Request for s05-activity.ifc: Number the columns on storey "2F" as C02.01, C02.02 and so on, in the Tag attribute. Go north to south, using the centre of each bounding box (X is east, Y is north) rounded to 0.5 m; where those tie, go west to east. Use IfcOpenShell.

First a look at what the model holds.

```python
import ifcopenshell
import ifcopenshell.util.element
import ifcopenshell.util.placement

model = ifcopenshell.open("s05-activity.ifc")
print(model.schema)
storey = next(s for s in model.by_type("IfcBuildingStorey") if s.Name == "2F")
columns = [e for e in ifcopenshell.util.element.get_decomposition(storey) if e.is_a("IfcColumn")]
for e in sorted(columns, key=lambda e: e.id()):
    origin = ifcopenshell.util.placement.get_local_placement(e.ObjectPlacement)[:3, 3]
    print(e.id(), e.Tag, e.Name, origin.round(2) + 0.0, sep=" | ")
```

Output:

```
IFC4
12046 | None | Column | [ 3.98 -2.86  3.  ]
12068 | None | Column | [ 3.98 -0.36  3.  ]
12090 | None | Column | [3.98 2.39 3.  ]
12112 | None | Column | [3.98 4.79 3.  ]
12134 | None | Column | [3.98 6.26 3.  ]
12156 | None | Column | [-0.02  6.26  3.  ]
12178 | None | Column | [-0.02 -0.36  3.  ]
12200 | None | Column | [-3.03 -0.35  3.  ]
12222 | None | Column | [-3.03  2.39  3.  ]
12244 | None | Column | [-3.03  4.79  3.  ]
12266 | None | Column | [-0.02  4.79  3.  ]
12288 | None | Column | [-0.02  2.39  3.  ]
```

```python
import ifcopenshell
import ifcopenshell.geom
import ifcopenshell.util.element
import ifcopenshell.util.shape

model = ifcopenshell.open("s05-activity.ifc")
settings = ifcopenshell.geom.settings()
settings.set("use-world-coords", True)


def centre(element):
    shape = ifcopenshell.geom.create_shape(settings, element)
    return ifcopenshell.util.shape.get_bbox_centroid(shape.geometry)


storey = next(s for s in model.by_type("IfcBuildingStorey") if s.Name == "2F")
columns = [e for e in ifcopenshell.util.element.get_decomposition(storey) if e.is_a("IfcColumn")]

# Insertion points can sit at a corner or the storey origin, so sort by the geometry (in metres).
centres = {e: centre(e) for e in columns}
columns.sort(key=lambda e: (-round(centres[e][1] / 0.5), centres[e][0]))

for i, e in enumerate(columns, start=1):
    number = f"C02.{i:02d}"
    e.Tag = number
    print(e.id(), number)

model.write("s05-activity_edited.ifc")
```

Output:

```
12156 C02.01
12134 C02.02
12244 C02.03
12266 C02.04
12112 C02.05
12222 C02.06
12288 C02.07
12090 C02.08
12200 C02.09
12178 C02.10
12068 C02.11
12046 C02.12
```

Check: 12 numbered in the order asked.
